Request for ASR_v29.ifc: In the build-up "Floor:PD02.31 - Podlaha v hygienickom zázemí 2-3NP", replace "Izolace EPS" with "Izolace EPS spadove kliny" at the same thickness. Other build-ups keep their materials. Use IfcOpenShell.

First a look at what the model holds.

```python
import ifcopenshell
import ifcopenshell.util.element

model = ifcopenshell.open("ASR_v29.ifc")
print(model.schema)
for layer_set in model.by_type("IfcMaterialLayerSet"):
    if layer_set.LayerSetName == "Floor:PD02.31 - Podlaha v hygienickom zázemí 2-3NP":
        for layer in layer_set.MaterialLayers:
            print(layer.id(), layer.Material and layer.Material.Name, layer.LayerThickness, sep=" | ")
        print(len(ifcopenshell.util.element.get_elements_by_material(model, layer_set)), "elements and types use it")
print(sorted(m.Name for m in model.by_type("IfcMaterial") if m.Name)[:60])
```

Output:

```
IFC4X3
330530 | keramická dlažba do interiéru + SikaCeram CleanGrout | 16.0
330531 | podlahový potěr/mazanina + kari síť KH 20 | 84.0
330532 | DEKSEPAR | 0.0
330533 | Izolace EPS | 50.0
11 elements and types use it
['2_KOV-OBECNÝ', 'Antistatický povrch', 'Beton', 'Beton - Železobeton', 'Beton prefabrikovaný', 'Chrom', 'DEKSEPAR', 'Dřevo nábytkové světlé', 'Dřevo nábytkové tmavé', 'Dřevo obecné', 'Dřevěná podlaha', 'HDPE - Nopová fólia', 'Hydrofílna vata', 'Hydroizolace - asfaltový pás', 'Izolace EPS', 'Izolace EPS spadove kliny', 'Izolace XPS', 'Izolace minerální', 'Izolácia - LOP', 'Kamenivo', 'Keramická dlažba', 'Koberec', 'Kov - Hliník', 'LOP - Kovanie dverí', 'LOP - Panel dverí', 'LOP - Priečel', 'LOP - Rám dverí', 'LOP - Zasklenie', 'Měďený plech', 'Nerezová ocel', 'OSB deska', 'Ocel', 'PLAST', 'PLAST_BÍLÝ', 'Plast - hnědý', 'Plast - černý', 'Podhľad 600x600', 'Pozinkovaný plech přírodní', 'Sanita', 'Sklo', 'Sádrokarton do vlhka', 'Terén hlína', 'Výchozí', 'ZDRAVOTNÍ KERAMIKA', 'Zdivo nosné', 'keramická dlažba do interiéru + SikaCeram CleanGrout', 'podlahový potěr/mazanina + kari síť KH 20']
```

```python
import ifcopenshell
import ifcopenshell.api.material

model = ifcopenshell.open("ASR_v29.ifc")

layer_set = next(s for s in model.by_type("IfcMaterialLayerSet") if s.LayerSetName == "Floor:PD02.31 - Podlaha v hygienickom zázemí 2-3NP")
layer = next(l for l in layer_set.MaterialLayers if l.Material and l.Material.Name == "Izolace EPS")
material = next(m for m in model.by_type("IfcMaterial") if m.Name == "Izolace EPS spadove kliny")

# Point this one layer at the other material; renaming the old one would change it everywhere.
ifcopenshell.api.material.edit_layer(model, layer=layer, attributes={"Name": material.Name}, material=material)

print([l.Material.Name if l.Material else None for l in layer_set.MaterialLayers])

model.write("ASR_v29-out.ifc")
```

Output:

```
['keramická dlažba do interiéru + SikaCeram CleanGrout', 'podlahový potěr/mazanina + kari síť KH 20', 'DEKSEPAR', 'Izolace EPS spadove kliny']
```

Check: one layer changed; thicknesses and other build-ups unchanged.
